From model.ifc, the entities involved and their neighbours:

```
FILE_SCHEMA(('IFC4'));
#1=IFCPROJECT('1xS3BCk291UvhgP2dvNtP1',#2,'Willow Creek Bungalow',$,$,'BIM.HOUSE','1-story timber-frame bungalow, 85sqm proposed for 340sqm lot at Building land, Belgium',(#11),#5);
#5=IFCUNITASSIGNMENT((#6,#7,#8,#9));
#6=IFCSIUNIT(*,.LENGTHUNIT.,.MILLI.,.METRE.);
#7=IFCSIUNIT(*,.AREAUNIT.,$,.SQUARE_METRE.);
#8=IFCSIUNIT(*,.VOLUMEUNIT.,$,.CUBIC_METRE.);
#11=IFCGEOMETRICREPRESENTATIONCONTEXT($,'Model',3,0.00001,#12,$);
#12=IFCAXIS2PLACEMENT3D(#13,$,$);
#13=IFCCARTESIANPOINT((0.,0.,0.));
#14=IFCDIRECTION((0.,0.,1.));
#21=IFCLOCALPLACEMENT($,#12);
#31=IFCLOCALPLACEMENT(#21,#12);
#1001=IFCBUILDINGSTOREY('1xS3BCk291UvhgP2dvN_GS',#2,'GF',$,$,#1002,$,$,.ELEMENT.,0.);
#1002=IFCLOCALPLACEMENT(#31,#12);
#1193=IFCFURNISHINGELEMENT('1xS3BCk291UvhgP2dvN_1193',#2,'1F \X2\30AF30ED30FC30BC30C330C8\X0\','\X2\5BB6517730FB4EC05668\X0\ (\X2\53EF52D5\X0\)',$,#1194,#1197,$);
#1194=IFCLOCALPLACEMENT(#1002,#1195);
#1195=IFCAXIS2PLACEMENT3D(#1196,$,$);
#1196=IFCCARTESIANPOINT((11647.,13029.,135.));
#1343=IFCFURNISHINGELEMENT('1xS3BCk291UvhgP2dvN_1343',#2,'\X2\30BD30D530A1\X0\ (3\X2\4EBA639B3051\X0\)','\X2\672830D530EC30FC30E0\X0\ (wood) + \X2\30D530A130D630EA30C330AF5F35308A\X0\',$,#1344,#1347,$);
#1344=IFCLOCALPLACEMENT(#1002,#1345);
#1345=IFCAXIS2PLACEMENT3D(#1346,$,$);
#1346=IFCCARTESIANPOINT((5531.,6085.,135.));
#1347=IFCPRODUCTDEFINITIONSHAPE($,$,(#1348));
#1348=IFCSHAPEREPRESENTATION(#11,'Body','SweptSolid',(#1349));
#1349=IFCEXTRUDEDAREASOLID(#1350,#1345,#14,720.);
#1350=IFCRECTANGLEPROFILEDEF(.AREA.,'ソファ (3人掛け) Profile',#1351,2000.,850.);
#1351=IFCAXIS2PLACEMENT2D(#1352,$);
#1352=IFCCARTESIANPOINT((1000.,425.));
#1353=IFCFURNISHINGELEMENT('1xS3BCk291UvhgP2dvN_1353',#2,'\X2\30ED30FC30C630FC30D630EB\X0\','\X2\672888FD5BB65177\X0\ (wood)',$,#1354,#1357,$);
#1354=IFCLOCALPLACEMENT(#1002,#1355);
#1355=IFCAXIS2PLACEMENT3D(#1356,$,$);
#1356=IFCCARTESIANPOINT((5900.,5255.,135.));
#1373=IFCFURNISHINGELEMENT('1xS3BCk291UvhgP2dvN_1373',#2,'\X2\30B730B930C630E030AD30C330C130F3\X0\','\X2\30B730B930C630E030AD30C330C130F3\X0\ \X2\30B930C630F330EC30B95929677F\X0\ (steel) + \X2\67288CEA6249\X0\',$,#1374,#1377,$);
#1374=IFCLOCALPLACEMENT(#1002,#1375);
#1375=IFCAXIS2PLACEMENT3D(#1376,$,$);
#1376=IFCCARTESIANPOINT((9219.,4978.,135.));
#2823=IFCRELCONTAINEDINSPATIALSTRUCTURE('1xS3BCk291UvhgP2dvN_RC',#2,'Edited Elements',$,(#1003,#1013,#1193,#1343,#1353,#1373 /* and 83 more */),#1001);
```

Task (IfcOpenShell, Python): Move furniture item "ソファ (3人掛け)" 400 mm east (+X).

```python
import ifcopenshell
import ifcopenshell.api.geometry
import ifcopenshell.util.placement
import ifcopenshell.util.unit

model = ifcopenshell.open("model.ifc")
unit_scale = ifcopenshell.util.unit.calculate_unit_scale(model)

item = model.by_id(1343)
matrix = ifcopenshell.util.placement.get_local_placement(item.ObjectPlacement)
matrix[0, 3] += 0.4 / unit_scale
ifcopenshell.api.geometry.edit_object_placement(model, product=item, matrix=matrix, is_si=False)

print(ifcopenshell.util.placement.get_local_placement(item.ObjectPlacement).round(3) + 0.0)

model.write("model_rev.ifc")
```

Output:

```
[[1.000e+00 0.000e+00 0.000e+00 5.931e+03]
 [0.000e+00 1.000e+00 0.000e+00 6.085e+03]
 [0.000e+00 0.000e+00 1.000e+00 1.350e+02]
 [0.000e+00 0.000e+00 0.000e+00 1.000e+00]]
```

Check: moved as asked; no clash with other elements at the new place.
